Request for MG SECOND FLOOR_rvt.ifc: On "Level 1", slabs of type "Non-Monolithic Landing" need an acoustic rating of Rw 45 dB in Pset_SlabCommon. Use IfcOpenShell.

First a look at what the model holds.

```python
import ifcopenshell
import ifcopenshell.util.element

model = ifcopenshell.open("MG SECOND FLOOR_rvt.ifc")
print(model.schema)
storey = next(s for s in model.by_type("IfcBuildingStorey") if s.Name == "Level 1")
slabs = [e for e in ifcopenshell.util.element.get_decomposition(storey) if e.is_a("IfcSlab")]
seen = {}
for e in slabs:
    element_type = ifcopenshell.util.element.get_type(e)
    key = (element_type.Name if element_type != e and element_type else None, ifcopenshell.util.element.get_pset(e, "Pset_SlabCommon", "AcousticRating"))
    seen[key] = seen.get(key, 0) + 1
for (name, value), count in sorted(seen.items(), key=str):
    print(count, "x", name, "|", value)
```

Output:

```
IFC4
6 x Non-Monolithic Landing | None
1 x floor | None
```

```python
import ifcopenshell
import ifcopenshell.api.pset
import ifcopenshell.util.element

model = ifcopenshell.open("MG SECOND FLOOR_rvt.ifc")

storey = next(s for s in model.by_type("IfcBuildingStorey") if s.Name == "Level 1")
slabs = [e for e in ifcopenshell.util.element.get_decomposition(storey) if e.is_a("IfcSlab")]

count = 0
for e in slabs:
    element_type = ifcopenshell.util.element.get_type(e)
    if element_type in (None, e) or element_type.Name != "Non-Monolithic Landing":
        continue
    # add_pset returns the element's existing set when there is one.
    pset = ifcopenshell.api.pset.add_pset(model, product=e, name="Pset_SlabCommon")
    ifcopenshell.api.pset.edit_pset(model, pset=pset, properties={"AcousticRating": "Rw 45 dB"})
    count += 1

print(count, "slabs updated")

model.write("MG SECOND FLOOR_rvt_v2.ifc")
```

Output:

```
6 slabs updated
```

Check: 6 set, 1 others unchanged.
